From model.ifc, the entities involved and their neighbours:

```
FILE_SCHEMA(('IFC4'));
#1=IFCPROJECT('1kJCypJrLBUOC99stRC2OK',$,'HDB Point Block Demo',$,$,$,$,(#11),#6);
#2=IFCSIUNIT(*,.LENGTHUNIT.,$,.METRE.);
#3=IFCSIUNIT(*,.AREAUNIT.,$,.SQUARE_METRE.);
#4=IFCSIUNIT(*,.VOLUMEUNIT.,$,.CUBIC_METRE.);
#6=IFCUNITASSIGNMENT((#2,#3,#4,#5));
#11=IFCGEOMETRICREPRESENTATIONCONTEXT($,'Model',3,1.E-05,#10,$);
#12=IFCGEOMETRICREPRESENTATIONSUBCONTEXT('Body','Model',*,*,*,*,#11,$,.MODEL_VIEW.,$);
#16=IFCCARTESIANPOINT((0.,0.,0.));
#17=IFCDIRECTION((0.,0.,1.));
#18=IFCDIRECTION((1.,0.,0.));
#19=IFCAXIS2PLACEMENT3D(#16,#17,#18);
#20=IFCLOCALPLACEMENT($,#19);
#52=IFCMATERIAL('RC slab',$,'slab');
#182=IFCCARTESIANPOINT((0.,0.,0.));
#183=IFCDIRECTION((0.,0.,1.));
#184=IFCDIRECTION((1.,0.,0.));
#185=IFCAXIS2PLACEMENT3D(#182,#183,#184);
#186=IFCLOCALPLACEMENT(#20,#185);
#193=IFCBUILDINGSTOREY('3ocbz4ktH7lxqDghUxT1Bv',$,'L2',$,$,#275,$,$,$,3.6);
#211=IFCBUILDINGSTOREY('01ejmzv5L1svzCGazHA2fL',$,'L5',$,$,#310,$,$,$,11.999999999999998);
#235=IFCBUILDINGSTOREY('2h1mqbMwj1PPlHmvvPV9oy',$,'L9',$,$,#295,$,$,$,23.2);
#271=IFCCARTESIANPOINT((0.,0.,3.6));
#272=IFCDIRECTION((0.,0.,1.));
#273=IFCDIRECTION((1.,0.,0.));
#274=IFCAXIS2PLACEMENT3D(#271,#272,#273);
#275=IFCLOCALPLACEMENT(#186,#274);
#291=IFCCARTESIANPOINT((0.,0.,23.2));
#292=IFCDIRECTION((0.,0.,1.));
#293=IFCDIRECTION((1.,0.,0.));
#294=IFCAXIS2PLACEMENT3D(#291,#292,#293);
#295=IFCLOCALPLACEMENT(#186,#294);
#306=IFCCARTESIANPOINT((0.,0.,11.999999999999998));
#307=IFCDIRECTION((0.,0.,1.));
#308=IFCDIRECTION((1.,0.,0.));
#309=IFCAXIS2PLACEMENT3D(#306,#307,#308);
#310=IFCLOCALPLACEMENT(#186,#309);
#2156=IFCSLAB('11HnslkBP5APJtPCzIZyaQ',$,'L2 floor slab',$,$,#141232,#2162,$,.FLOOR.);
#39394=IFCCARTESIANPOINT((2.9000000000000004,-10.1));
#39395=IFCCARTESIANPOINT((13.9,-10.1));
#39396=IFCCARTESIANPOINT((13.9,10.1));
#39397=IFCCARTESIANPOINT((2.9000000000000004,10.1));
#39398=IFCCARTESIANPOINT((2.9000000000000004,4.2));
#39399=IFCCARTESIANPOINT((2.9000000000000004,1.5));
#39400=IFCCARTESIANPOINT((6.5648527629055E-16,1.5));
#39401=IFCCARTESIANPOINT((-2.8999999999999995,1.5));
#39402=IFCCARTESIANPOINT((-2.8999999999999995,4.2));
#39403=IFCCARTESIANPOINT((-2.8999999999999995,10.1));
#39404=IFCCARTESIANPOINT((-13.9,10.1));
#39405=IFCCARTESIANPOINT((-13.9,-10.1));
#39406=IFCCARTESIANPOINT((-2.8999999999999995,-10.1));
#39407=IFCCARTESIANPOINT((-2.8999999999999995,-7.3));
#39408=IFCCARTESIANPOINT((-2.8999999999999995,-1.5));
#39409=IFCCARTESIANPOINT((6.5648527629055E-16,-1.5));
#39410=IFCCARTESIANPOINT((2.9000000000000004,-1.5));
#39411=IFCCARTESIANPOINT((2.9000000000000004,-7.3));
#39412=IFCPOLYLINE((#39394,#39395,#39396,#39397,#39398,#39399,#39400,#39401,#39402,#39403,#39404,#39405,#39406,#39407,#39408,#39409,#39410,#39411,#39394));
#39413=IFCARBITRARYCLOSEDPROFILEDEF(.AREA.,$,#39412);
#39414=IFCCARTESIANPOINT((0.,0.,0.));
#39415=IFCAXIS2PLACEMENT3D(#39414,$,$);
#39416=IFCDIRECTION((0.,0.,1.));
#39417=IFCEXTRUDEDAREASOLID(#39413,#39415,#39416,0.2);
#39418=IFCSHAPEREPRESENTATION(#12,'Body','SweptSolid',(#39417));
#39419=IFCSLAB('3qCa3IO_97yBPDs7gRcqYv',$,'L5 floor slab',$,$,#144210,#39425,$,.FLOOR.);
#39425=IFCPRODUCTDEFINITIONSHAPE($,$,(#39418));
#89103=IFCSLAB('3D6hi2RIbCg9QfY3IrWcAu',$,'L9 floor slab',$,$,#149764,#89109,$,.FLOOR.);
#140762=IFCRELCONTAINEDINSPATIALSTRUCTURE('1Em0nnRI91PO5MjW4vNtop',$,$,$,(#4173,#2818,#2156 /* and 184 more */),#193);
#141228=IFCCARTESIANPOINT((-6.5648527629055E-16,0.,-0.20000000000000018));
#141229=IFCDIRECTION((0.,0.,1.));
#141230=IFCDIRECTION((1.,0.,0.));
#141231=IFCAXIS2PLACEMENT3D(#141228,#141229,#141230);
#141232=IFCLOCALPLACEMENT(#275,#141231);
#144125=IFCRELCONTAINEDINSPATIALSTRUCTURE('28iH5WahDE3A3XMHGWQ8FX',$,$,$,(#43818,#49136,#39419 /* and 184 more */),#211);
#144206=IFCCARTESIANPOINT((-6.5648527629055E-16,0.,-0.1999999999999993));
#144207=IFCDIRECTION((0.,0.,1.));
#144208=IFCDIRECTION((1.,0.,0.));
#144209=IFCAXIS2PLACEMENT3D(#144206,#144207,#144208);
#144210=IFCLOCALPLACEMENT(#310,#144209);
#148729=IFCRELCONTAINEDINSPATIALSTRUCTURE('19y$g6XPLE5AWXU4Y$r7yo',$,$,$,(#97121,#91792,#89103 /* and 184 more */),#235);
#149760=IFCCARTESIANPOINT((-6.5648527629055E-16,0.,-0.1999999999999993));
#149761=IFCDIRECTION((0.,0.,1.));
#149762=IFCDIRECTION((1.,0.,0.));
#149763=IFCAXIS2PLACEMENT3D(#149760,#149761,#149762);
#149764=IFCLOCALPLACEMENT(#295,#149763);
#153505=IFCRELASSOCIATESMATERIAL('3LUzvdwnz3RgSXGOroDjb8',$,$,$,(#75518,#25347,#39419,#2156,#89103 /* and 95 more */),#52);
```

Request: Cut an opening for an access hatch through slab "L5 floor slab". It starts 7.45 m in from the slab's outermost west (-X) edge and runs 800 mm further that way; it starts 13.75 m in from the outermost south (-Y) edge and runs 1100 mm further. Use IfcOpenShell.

```python
import numpy as np
import ifcopenshell
import ifcopenshell.api.feature
import ifcopenshell.api.geometry
import ifcopenshell.api.root
import ifcopenshell.geom
import ifcopenshell.util.placement
import ifcopenshell.util.representation
import ifcopenshell.util.shape
import ifcopenshell.util.unit

model = ifcopenshell.open("model.ifc")
unit_scale = ifcopenshell.util.unit.calculate_unit_scale(model)
settings = ifcopenshell.geom.settings()


def volume(element):
    """Net volume in cubic metres, openings subtracted."""
    shape = ifcopenshell.geom.create_shape(settings, element)
    return ifcopenshell.util.shape.get_volume(shape.geometry)


slab = model.by_guid("3qCa3IO_97yBPDs7gRcqYv")
before = volume(slab)

# Extent in the slab's own axes, in metres. The edges named are its -X and -Y sides.
slab_shape = ifcopenshell.geom.create_shape(settings, slab)
vertices = ifcopenshell.util.shape.get_vertices(slab_shape.geometry)
x_min, y_min, bottom = vertices.min(axis=0)
top = vertices[:, 2].max()

opening = ifcopenshell.api.root.create_entity(model, ifc_class="IfcOpeningElement", name="Access hatch opening", predefined_type="OPENING")
context = ifcopenshell.util.representation.get_context(model, "Model", "Body", "MODEL_VIEW")
width, depth = 0.8, 1.1
outline = [(0.0, 0.0), (width, 0.0), (width, depth), (0.0, depth), (0.0, 0.0)]
# Overshoot both faces by 50 mm so the cut is clean.
shape = ifcopenshell.api.geometry.add_slab_representation(
    model, context=context, depth=top - bottom + 0.1, polyline=outline
)
ifcopenshell.api.geometry.assign_representation(model, product=opening, representation=shape)

matrix = ifcopenshell.util.placement.get_local_placement(slab.ObjectPlacement)
matrix[:, 3] = matrix @ np.append(np.array([x_min + 7.45, y_min + 13.75, bottom - 0.05]) / unit_scale, 1.0)
ifcopenshell.api.geometry.edit_object_placement(model, product=opening, matrix=matrix, is_si=False)
ifcopenshell.api.feature.add_feature(model, feature=opening, element=slab)

after = volume(slab)

print(f"slab volume {before:.3f} -> {after:.3f} m3")

model.write("model_v2.ifc")
```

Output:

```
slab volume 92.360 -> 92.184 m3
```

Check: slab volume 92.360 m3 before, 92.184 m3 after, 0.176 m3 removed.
